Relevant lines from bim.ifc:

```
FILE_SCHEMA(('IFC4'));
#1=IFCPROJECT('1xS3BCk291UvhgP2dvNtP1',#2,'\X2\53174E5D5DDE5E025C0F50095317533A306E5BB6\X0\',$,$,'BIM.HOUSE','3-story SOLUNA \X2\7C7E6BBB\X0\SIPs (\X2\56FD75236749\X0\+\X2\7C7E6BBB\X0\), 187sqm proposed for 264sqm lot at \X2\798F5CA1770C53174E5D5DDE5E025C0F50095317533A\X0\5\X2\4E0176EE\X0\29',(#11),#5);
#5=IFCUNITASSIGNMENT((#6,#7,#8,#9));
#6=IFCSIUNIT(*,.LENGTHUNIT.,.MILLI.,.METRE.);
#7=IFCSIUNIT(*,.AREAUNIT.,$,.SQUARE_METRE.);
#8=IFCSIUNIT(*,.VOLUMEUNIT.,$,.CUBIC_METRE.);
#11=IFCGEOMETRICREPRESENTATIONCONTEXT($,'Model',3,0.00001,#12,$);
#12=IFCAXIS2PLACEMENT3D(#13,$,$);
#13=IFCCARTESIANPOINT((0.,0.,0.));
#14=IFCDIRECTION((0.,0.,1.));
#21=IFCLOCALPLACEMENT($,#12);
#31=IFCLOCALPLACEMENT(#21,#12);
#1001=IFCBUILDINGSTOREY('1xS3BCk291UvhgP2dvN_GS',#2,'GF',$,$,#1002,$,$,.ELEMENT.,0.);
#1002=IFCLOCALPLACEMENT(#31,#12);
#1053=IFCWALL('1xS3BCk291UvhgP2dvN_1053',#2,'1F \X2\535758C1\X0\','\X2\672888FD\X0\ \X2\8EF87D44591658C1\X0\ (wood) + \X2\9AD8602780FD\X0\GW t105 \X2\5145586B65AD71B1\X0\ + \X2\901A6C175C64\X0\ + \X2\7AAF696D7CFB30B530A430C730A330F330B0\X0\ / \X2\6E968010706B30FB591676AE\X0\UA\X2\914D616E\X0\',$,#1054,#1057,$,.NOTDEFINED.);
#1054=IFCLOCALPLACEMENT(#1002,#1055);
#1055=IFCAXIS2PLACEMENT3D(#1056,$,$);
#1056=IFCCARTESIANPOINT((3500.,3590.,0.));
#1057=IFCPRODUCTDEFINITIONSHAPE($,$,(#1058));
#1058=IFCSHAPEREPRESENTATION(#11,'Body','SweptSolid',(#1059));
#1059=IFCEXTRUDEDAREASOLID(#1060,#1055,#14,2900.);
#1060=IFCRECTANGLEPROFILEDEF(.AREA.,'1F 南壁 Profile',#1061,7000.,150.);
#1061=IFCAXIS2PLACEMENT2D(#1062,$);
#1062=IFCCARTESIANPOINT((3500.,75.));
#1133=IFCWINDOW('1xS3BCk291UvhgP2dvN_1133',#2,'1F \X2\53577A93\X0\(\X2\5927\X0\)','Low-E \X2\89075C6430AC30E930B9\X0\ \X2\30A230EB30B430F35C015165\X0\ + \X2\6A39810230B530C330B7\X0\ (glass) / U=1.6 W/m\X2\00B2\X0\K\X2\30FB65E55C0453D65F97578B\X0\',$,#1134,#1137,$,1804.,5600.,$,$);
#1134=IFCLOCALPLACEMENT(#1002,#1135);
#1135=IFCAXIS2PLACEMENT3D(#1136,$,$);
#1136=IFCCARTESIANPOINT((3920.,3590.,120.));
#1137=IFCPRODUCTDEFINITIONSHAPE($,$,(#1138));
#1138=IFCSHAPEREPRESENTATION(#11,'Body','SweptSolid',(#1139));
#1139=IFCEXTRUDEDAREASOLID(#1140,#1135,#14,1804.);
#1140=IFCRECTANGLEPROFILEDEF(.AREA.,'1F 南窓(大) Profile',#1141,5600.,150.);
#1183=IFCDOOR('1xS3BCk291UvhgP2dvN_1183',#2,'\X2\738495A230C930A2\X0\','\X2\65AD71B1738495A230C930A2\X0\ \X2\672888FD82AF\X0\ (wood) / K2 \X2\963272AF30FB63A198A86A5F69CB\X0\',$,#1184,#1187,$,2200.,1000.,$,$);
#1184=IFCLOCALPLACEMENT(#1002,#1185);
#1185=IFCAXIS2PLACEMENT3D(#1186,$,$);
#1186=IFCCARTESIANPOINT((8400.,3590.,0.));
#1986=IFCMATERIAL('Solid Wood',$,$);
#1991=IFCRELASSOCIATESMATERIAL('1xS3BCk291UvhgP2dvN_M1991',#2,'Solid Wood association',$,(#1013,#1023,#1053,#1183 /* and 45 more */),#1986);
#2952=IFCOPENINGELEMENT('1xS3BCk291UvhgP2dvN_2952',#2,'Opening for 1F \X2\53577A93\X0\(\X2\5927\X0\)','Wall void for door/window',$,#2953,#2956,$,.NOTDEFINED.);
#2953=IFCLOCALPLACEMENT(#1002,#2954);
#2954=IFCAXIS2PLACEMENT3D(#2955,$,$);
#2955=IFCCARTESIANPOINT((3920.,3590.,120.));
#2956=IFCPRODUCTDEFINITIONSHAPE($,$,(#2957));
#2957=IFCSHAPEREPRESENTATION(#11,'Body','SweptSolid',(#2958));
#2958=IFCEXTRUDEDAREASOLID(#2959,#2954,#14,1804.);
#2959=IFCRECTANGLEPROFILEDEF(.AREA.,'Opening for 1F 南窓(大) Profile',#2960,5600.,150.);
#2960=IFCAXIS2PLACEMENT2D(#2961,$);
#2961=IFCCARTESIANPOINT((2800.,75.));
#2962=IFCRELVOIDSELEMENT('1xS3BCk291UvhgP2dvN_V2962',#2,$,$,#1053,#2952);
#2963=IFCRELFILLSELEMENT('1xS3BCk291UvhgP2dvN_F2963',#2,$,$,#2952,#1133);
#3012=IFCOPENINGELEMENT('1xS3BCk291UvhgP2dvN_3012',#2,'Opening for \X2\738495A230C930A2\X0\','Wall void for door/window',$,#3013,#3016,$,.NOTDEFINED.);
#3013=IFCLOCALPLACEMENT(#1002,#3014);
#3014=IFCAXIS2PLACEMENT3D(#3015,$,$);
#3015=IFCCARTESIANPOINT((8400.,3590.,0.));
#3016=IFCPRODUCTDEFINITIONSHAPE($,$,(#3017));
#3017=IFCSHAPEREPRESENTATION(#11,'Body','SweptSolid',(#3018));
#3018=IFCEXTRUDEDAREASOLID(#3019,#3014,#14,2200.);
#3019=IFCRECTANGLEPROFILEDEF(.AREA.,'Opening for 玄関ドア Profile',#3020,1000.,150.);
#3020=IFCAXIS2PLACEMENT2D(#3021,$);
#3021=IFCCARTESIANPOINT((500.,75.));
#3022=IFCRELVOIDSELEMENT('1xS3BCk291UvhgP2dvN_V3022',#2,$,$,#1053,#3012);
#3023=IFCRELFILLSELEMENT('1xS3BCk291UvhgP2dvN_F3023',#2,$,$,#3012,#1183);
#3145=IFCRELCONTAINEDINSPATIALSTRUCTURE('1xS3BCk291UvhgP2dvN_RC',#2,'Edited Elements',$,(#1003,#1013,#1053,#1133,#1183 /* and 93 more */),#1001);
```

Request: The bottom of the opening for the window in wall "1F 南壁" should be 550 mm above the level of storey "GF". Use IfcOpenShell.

```python
import numpy as np
import ifcopenshell
import ifcopenshell.api.geometry
import ifcopenshell.geom
import ifcopenshell.util.element
import ifcopenshell.util.placement
import ifcopenshell.util.shape
import ifcopenshell.util.unit

model = ifcopenshell.open("bim.ifc")
unit_scale = ifcopenshell.util.unit.calculate_unit_scale(model)

window = model.by_guid("1xS3BCk291UvhgP2dvN_1133")
opening = window.FillsVoids[0].RelatingOpeningElement
storey = ifcopenshell.util.element.get_container(window, ifc_class="IfcBuildingStorey")
level = ifcopenshell.util.placement.get_local_placement(storey.ObjectPlacement)[2, 3]

# The opening's origin need not be at the sill, so measure its lowest point.
shape = ifcopenshell.geom.create_shape(ifcopenshell.geom.settings(), opening)
bottom = ifcopenshell.util.shape.get_shape_bottom_elevation(shape, shape.geometry) / unit_scale
dz = level + 550.0 - bottom

shift = np.array([0.0, 0.0, dz])
# The window is not placed relative to its opening, so move both.
for product in (opening, window):
    matrix = ifcopenshell.util.placement.get_local_placement(product.ObjectPlacement)
    matrix[:3, 3] += shift
    ifcopenshell.api.geometry.edit_object_placement(model, product=product, matrix=matrix, is_si=False)

print(f"moved by {dz * unit_scale:+.3f} m")

model.write("bim_updated.ifc")
```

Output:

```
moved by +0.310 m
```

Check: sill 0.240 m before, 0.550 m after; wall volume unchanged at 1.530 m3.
